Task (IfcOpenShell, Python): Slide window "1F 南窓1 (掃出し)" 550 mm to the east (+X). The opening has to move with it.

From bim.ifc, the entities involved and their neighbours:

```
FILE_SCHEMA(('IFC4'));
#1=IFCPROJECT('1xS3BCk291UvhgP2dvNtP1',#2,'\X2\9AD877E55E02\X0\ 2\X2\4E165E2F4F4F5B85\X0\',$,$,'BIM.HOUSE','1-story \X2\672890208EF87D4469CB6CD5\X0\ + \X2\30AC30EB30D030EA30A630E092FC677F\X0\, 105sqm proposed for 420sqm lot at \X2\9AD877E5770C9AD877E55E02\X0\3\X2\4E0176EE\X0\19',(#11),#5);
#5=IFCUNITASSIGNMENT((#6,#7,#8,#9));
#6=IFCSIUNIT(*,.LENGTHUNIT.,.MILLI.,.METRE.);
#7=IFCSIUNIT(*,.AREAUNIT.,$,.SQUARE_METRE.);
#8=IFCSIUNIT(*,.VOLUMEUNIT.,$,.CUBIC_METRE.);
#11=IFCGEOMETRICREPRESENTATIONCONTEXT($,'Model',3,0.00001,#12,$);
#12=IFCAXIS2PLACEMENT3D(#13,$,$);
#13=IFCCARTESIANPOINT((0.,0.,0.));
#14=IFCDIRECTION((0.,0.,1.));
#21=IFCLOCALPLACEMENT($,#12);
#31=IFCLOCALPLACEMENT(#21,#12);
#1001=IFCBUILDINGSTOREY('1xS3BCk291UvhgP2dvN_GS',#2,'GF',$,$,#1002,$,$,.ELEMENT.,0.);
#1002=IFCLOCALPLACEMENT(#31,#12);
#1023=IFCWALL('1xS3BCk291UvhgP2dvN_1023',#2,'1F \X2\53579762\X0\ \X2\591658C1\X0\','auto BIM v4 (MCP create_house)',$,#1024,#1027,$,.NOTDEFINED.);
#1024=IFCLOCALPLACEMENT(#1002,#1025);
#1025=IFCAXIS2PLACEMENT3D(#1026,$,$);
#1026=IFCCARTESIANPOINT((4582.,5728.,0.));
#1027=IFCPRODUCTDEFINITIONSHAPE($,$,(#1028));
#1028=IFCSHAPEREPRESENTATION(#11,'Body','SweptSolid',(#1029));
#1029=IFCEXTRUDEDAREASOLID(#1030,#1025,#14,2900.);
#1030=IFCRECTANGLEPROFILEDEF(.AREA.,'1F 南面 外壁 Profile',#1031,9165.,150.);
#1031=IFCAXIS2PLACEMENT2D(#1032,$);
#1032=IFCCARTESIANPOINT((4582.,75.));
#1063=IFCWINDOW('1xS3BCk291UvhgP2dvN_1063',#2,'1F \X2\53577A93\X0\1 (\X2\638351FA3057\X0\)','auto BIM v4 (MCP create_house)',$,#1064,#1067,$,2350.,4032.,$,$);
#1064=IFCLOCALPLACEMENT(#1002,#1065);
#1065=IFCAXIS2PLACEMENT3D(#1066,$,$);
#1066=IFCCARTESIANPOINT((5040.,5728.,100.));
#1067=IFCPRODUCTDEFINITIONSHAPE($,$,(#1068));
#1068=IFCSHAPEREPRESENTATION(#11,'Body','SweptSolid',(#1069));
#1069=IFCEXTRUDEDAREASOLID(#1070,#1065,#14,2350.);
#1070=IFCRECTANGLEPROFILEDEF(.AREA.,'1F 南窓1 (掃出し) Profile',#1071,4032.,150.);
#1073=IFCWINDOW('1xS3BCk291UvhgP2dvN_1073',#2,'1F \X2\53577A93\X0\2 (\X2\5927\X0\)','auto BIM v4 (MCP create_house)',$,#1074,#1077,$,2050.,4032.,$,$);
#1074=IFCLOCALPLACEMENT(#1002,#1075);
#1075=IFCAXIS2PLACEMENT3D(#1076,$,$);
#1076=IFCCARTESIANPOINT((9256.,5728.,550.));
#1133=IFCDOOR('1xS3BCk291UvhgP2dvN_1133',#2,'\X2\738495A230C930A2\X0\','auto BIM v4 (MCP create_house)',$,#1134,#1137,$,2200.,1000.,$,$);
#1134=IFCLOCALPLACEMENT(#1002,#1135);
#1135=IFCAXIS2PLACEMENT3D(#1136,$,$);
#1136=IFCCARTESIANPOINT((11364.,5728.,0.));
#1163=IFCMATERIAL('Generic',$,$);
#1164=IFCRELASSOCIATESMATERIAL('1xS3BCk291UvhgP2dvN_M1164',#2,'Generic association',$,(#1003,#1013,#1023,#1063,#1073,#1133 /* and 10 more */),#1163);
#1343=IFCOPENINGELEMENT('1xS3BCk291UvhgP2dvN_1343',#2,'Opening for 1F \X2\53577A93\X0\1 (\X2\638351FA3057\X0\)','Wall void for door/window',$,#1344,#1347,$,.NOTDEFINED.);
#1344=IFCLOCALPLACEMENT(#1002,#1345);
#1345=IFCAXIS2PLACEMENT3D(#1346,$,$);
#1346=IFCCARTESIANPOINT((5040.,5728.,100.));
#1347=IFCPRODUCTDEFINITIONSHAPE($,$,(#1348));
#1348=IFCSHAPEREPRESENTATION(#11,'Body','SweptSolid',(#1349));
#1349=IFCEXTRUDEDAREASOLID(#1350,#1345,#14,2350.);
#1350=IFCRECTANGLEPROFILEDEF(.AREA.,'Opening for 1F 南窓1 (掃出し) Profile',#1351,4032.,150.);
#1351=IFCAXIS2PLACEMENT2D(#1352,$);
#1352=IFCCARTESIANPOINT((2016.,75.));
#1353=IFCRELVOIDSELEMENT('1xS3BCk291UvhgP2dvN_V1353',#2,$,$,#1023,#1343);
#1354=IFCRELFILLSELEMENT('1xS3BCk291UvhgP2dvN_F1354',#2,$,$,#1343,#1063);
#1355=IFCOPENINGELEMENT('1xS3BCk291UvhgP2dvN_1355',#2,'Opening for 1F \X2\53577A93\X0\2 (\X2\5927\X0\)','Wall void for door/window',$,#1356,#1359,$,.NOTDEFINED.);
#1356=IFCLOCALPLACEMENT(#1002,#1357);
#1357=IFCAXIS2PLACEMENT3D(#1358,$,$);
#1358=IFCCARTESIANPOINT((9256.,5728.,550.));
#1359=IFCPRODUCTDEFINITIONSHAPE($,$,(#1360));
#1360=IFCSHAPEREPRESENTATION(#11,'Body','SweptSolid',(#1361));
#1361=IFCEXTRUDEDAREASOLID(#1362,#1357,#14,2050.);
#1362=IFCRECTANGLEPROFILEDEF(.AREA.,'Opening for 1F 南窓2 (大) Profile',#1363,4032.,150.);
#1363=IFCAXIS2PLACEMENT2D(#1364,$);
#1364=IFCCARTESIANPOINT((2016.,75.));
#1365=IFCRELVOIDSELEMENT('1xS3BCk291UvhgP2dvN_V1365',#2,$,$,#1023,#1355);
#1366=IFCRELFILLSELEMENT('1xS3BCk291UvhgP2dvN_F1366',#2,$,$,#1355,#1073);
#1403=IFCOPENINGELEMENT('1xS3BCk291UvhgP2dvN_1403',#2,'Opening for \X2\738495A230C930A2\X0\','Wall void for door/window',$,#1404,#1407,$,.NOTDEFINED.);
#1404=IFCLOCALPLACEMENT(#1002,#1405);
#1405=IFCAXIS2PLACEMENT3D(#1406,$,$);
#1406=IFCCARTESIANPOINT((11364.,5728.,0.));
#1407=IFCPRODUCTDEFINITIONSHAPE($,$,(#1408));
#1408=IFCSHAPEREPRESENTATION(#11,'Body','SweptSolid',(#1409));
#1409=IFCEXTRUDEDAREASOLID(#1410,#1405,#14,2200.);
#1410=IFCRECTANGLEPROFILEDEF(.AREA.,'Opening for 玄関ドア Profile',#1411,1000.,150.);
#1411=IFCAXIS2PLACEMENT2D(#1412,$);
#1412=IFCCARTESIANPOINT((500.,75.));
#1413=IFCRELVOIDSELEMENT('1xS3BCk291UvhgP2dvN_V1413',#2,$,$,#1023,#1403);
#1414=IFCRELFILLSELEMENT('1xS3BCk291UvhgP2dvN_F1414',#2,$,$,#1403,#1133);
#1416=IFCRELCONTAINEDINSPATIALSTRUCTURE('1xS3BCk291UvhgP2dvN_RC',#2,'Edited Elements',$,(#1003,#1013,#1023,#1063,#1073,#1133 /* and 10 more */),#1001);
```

```python
import ifcopenshell
import ifcopenshell.api.geometry
import ifcopenshell.util.placement

model = ifcopenshell.open("bim.ifc")

window = model.by_guid("1xS3BCk291UvhgP2dvN_1063")
opening = window.FillsVoids[0].RelatingOpeningElement
wall = opening.VoidsElements[0].RelatingBuildingElement

wall_matrix = ifcopenshell.util.placement.get_local_placement(wall.ObjectPlacement)
shift = wall_matrix[:3, 0] * 550.0
before = ifcopenshell.util.placement.get_local_placement(window.ObjectPlacement)[:3, 3].copy()

# The window is not placed relative to its opening, so move both.
for product in (opening, window):
    matrix = ifcopenshell.util.placement.get_local_placement(product.ObjectPlacement)
    matrix[:3, 3] += shift
    ifcopenshell.api.geometry.edit_object_placement(model, product=product, matrix=matrix, is_si=False)

after = ifcopenshell.util.placement.get_local_placement(window.ObjectPlacement)[:3, 3]
print("window moved by", (after - before).round(3) + 0.0)

model.write("bim_edited.ifc")
```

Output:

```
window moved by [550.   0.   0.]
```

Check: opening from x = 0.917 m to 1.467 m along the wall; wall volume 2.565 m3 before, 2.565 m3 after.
